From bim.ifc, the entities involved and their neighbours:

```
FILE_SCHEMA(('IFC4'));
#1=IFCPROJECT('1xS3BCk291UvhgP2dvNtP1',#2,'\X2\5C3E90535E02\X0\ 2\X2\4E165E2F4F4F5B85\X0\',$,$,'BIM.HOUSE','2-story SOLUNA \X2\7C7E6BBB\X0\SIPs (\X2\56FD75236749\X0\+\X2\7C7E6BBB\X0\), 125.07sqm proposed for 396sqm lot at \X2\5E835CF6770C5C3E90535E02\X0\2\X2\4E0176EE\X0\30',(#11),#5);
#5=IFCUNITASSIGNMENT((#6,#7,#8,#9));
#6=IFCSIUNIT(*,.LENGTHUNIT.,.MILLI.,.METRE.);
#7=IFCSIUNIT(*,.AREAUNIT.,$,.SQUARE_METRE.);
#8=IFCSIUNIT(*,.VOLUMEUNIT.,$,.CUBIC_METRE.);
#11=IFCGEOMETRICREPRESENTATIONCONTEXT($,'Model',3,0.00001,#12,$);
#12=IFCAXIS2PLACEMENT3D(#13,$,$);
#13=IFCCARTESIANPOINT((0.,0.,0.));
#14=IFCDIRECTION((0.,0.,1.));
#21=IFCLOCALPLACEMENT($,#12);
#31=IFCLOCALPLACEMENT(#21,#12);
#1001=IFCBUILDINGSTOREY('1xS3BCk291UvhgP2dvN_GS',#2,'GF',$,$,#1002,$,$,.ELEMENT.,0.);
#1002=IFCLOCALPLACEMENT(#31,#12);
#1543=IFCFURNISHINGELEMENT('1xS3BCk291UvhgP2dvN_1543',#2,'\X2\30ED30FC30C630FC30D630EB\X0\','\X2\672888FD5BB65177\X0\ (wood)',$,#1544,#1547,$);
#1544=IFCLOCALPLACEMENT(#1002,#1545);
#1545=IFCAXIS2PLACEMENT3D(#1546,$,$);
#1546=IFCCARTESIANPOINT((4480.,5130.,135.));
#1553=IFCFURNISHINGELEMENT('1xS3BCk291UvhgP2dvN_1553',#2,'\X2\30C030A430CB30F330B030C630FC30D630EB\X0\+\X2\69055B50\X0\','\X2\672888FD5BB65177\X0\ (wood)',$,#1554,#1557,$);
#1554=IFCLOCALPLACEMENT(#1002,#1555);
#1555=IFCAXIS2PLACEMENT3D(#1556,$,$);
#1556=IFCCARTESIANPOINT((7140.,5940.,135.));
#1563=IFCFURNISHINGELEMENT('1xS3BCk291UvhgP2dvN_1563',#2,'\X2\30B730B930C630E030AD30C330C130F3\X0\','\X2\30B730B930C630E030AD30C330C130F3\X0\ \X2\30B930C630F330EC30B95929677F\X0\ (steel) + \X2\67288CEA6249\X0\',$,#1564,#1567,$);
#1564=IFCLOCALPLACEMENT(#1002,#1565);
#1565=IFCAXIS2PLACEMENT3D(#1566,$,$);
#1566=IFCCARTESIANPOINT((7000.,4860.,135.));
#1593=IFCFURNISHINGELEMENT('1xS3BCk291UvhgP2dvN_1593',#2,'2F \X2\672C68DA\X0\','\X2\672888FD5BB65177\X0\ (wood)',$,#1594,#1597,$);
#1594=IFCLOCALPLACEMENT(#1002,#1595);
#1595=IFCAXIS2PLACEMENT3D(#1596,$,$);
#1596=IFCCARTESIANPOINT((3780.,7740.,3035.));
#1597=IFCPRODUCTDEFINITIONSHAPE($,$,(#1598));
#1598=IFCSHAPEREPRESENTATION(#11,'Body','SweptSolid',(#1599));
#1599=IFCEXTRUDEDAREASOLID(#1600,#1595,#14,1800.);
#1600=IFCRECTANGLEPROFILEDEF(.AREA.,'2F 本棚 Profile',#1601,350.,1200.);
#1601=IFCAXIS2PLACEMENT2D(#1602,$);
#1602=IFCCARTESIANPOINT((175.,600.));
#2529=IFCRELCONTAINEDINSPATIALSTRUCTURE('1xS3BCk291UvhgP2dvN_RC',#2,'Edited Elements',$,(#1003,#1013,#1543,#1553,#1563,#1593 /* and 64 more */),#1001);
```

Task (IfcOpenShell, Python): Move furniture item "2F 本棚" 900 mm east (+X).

```python
import ifcopenshell
import ifcopenshell.api.geometry
import ifcopenshell.util.placement

model = ifcopenshell.open("bim.ifc")

item = model.by_guid("1xS3BCk291UvhgP2dvN_1593")
matrix = ifcopenshell.util.placement.get_local_placement(item.ObjectPlacement)
matrix[0, 3] += 900.0
ifcopenshell.api.geometry.edit_object_placement(model, product=item, matrix=matrix, is_si=False)

print(ifcopenshell.util.placement.get_local_placement(item.ObjectPlacement).round(3) + 0.0)

model.write("bim-out.ifc")
```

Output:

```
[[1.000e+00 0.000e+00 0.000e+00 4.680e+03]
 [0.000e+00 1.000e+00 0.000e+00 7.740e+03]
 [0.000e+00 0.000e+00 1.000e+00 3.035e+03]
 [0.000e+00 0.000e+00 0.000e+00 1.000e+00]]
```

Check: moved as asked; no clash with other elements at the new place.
